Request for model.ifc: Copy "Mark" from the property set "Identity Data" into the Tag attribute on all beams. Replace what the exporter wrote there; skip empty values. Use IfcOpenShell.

First a look at what the model holds.

```python
import ifcopenshell
import ifcopenshell.util.element

model = ifcopenshell.open("model.ifc")
print(model.schema)
beams = model.by_type("IfcBeam")
print(len(beams), "beams")
for e in beams[:8]:
    source = ifcopenshell.util.element.get_pset(e, "Identity Data", "Mark")
    target = e.Tag
    print(e.id(), repr(source), repr(target), sep=" | ")
```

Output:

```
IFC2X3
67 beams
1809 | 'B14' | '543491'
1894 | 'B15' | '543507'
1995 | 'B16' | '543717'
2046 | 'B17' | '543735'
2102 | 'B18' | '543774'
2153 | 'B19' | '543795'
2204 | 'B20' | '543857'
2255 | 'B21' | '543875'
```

```python
import ifcopenshell
import ifcopenshell.util.element

model = ifcopenshell.open("model.ifc")

count = 0
for e in model.by_type("IfcBeam"):
    value = ifcopenshell.util.element.get_pset(e, "Identity Data", "Mark")
    current = e.Tag
    if not value or not value.strip() or current == value:
        continue
    e.Tag = value
    count += 1

print(count, "beams updated")

model.write("model_edited.ifc")
```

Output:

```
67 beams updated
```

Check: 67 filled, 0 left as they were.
